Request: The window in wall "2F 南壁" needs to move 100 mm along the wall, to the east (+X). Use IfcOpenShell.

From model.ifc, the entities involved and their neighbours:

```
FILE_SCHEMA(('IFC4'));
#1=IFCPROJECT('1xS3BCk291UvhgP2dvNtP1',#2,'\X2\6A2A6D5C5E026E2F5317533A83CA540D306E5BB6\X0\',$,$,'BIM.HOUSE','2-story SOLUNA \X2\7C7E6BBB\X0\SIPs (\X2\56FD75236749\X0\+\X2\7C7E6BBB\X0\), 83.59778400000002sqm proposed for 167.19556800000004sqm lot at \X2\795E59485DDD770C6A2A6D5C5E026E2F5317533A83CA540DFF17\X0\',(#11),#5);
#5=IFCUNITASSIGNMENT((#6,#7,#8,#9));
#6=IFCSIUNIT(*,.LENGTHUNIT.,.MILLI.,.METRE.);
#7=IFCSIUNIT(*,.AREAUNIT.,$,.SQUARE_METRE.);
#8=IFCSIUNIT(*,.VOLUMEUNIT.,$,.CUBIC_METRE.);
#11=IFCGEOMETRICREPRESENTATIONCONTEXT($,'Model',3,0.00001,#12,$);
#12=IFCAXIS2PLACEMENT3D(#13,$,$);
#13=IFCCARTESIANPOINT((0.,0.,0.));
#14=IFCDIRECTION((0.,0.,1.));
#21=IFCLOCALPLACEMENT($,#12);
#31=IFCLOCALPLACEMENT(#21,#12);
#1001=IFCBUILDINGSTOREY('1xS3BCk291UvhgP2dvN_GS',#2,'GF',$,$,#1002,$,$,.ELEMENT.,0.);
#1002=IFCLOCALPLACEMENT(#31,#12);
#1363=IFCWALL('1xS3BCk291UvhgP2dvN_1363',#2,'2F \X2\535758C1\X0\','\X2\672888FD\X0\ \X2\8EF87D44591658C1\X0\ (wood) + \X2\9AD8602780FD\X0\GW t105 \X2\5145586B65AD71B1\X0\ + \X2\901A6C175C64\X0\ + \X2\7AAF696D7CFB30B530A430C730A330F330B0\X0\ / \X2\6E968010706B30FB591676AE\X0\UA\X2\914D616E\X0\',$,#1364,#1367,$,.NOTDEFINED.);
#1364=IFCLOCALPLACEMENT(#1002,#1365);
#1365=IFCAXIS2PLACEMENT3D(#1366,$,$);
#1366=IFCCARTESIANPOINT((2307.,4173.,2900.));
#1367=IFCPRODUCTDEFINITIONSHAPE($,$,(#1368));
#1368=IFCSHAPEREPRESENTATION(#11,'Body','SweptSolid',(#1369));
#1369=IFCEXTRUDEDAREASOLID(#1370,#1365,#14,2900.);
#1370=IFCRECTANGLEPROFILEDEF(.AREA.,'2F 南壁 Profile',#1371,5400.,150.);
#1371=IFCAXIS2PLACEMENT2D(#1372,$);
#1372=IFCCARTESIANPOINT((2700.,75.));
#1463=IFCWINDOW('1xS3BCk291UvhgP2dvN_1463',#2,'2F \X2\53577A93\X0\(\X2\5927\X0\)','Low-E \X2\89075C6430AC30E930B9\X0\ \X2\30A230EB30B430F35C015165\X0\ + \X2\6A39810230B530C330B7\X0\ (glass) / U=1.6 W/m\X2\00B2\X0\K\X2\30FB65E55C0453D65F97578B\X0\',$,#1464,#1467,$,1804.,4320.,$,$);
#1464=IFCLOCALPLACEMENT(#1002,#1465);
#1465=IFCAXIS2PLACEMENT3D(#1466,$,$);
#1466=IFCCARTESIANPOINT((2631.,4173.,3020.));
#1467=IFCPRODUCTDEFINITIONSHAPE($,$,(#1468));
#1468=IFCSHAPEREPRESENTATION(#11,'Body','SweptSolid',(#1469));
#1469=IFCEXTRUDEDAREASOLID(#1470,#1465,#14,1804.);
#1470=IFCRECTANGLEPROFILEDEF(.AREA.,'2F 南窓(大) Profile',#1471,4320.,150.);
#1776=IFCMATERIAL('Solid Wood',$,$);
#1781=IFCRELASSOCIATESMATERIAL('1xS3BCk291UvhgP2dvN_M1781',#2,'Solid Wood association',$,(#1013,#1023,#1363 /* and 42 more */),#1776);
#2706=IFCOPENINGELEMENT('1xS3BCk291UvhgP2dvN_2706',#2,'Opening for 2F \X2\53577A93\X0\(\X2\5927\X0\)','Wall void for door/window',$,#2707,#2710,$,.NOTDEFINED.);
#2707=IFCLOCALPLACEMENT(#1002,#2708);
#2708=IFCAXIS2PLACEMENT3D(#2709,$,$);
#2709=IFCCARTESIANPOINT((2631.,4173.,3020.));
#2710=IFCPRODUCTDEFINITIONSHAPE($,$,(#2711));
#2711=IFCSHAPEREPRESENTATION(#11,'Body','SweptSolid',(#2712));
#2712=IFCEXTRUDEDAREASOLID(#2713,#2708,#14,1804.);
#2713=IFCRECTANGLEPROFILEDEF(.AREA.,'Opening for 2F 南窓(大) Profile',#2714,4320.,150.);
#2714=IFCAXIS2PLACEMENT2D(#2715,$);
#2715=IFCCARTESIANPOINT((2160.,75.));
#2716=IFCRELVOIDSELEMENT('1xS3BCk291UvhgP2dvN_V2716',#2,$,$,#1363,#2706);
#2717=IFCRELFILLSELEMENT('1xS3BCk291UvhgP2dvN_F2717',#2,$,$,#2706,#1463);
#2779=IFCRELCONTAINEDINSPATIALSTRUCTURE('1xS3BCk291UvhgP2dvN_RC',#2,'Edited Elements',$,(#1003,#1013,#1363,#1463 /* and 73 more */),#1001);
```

```python
import ifcopenshell
import ifcopenshell.api.geometry
import ifcopenshell.util.placement
import ifcopenshell.util.unit

model = ifcopenshell.open("model.ifc")
unit_scale = ifcopenshell.util.unit.calculate_unit_scale(model)

window = model.by_id(1463)
opening = window.FillsVoids[0].RelatingOpeningElement
wall = opening.VoidsElements[0].RelatingBuildingElement

wall_matrix = ifcopenshell.util.placement.get_local_placement(wall.ObjectPlacement)
shift = wall_matrix[:3, 0] * 0.1 / unit_scale
before = ifcopenshell.util.placement.get_local_placement(window.ObjectPlacement)[:3, 3].copy()

# The window is not placed relative to its opening, so move both.
for product in (opening, window):
    matrix = ifcopenshell.util.placement.get_local_placement(product.ObjectPlacement)
    matrix[:3, 3] += shift
    ifcopenshell.api.geometry.edit_object_placement(model, product=product, matrix=matrix, is_si=False)

after = ifcopenshell.util.placement.get_local_placement(window.ObjectPlacement)[:3, 3]
print("window moved by", (after - before).round(3) + 0.0)

model.write("model-out.ifc")
```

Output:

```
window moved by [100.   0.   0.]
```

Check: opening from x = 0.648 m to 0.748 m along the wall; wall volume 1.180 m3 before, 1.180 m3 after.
